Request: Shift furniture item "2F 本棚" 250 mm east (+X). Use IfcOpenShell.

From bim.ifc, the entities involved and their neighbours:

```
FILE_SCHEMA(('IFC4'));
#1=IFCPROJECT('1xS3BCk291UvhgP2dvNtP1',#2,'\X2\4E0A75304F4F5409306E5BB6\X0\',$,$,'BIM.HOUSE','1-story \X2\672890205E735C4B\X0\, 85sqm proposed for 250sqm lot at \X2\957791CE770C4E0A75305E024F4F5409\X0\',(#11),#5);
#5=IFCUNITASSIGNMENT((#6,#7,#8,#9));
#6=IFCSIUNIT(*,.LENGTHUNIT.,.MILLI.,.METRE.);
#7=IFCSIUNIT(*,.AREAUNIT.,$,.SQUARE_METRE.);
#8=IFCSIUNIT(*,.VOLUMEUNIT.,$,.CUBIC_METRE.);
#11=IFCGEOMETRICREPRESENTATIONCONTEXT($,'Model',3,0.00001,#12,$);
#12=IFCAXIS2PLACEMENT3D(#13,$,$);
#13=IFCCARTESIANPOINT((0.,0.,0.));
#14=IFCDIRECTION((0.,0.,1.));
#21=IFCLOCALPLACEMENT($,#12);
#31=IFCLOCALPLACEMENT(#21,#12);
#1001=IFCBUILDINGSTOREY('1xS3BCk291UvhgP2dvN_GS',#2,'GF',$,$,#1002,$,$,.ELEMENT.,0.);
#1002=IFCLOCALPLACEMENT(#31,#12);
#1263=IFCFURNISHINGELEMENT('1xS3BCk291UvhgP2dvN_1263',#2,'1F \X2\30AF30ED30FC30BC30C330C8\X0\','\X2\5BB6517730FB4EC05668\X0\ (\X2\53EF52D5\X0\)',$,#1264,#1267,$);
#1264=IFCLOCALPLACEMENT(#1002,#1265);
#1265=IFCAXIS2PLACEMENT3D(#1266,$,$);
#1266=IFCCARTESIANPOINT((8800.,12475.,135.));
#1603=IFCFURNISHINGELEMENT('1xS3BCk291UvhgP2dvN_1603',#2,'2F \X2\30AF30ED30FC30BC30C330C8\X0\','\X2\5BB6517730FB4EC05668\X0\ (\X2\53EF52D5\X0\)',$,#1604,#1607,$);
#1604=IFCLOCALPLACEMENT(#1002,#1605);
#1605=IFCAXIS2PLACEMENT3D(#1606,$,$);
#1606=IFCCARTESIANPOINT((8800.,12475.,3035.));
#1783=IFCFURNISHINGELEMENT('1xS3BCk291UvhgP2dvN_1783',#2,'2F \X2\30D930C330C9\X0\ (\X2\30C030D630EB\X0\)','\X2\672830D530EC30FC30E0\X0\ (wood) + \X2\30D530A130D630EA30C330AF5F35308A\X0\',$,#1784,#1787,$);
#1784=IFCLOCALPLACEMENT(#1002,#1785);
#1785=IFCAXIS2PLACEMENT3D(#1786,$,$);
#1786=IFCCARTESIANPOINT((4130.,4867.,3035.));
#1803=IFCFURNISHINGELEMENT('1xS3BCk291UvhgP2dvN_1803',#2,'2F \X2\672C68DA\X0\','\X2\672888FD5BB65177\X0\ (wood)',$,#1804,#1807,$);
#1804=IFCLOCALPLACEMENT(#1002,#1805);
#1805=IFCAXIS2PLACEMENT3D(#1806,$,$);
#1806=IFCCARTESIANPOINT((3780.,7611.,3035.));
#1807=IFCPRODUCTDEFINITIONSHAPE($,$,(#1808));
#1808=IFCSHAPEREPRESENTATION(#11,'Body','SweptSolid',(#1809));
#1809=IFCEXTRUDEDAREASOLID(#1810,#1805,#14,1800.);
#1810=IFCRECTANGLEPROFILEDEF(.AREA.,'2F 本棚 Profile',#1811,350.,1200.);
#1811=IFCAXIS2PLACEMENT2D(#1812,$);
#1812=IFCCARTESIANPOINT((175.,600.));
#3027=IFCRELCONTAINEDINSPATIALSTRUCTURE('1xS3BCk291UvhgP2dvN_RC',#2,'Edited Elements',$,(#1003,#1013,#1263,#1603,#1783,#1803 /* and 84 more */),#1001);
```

```python
import ifcopenshell
import ifcopenshell.api.geometry
import ifcopenshell.util.placement
import ifcopenshell.util.unit

model = ifcopenshell.open("bim.ifc")
unit_scale = ifcopenshell.util.unit.calculate_unit_scale(model)

item = model.by_id(1803)
matrix = ifcopenshell.util.placement.get_local_placement(item.ObjectPlacement)
matrix[0, 3] += 0.25 / unit_scale
ifcopenshell.api.geometry.edit_object_placement(model, product=item, matrix=matrix, is_si=False)

print(ifcopenshell.util.placement.get_local_placement(item.ObjectPlacement).round(3) + 0.0)

model.write("bim_updated.ifc")
```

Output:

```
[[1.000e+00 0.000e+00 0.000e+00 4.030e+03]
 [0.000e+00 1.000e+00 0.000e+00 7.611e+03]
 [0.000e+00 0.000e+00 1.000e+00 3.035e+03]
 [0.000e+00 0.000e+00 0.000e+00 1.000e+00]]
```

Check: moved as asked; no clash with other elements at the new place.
